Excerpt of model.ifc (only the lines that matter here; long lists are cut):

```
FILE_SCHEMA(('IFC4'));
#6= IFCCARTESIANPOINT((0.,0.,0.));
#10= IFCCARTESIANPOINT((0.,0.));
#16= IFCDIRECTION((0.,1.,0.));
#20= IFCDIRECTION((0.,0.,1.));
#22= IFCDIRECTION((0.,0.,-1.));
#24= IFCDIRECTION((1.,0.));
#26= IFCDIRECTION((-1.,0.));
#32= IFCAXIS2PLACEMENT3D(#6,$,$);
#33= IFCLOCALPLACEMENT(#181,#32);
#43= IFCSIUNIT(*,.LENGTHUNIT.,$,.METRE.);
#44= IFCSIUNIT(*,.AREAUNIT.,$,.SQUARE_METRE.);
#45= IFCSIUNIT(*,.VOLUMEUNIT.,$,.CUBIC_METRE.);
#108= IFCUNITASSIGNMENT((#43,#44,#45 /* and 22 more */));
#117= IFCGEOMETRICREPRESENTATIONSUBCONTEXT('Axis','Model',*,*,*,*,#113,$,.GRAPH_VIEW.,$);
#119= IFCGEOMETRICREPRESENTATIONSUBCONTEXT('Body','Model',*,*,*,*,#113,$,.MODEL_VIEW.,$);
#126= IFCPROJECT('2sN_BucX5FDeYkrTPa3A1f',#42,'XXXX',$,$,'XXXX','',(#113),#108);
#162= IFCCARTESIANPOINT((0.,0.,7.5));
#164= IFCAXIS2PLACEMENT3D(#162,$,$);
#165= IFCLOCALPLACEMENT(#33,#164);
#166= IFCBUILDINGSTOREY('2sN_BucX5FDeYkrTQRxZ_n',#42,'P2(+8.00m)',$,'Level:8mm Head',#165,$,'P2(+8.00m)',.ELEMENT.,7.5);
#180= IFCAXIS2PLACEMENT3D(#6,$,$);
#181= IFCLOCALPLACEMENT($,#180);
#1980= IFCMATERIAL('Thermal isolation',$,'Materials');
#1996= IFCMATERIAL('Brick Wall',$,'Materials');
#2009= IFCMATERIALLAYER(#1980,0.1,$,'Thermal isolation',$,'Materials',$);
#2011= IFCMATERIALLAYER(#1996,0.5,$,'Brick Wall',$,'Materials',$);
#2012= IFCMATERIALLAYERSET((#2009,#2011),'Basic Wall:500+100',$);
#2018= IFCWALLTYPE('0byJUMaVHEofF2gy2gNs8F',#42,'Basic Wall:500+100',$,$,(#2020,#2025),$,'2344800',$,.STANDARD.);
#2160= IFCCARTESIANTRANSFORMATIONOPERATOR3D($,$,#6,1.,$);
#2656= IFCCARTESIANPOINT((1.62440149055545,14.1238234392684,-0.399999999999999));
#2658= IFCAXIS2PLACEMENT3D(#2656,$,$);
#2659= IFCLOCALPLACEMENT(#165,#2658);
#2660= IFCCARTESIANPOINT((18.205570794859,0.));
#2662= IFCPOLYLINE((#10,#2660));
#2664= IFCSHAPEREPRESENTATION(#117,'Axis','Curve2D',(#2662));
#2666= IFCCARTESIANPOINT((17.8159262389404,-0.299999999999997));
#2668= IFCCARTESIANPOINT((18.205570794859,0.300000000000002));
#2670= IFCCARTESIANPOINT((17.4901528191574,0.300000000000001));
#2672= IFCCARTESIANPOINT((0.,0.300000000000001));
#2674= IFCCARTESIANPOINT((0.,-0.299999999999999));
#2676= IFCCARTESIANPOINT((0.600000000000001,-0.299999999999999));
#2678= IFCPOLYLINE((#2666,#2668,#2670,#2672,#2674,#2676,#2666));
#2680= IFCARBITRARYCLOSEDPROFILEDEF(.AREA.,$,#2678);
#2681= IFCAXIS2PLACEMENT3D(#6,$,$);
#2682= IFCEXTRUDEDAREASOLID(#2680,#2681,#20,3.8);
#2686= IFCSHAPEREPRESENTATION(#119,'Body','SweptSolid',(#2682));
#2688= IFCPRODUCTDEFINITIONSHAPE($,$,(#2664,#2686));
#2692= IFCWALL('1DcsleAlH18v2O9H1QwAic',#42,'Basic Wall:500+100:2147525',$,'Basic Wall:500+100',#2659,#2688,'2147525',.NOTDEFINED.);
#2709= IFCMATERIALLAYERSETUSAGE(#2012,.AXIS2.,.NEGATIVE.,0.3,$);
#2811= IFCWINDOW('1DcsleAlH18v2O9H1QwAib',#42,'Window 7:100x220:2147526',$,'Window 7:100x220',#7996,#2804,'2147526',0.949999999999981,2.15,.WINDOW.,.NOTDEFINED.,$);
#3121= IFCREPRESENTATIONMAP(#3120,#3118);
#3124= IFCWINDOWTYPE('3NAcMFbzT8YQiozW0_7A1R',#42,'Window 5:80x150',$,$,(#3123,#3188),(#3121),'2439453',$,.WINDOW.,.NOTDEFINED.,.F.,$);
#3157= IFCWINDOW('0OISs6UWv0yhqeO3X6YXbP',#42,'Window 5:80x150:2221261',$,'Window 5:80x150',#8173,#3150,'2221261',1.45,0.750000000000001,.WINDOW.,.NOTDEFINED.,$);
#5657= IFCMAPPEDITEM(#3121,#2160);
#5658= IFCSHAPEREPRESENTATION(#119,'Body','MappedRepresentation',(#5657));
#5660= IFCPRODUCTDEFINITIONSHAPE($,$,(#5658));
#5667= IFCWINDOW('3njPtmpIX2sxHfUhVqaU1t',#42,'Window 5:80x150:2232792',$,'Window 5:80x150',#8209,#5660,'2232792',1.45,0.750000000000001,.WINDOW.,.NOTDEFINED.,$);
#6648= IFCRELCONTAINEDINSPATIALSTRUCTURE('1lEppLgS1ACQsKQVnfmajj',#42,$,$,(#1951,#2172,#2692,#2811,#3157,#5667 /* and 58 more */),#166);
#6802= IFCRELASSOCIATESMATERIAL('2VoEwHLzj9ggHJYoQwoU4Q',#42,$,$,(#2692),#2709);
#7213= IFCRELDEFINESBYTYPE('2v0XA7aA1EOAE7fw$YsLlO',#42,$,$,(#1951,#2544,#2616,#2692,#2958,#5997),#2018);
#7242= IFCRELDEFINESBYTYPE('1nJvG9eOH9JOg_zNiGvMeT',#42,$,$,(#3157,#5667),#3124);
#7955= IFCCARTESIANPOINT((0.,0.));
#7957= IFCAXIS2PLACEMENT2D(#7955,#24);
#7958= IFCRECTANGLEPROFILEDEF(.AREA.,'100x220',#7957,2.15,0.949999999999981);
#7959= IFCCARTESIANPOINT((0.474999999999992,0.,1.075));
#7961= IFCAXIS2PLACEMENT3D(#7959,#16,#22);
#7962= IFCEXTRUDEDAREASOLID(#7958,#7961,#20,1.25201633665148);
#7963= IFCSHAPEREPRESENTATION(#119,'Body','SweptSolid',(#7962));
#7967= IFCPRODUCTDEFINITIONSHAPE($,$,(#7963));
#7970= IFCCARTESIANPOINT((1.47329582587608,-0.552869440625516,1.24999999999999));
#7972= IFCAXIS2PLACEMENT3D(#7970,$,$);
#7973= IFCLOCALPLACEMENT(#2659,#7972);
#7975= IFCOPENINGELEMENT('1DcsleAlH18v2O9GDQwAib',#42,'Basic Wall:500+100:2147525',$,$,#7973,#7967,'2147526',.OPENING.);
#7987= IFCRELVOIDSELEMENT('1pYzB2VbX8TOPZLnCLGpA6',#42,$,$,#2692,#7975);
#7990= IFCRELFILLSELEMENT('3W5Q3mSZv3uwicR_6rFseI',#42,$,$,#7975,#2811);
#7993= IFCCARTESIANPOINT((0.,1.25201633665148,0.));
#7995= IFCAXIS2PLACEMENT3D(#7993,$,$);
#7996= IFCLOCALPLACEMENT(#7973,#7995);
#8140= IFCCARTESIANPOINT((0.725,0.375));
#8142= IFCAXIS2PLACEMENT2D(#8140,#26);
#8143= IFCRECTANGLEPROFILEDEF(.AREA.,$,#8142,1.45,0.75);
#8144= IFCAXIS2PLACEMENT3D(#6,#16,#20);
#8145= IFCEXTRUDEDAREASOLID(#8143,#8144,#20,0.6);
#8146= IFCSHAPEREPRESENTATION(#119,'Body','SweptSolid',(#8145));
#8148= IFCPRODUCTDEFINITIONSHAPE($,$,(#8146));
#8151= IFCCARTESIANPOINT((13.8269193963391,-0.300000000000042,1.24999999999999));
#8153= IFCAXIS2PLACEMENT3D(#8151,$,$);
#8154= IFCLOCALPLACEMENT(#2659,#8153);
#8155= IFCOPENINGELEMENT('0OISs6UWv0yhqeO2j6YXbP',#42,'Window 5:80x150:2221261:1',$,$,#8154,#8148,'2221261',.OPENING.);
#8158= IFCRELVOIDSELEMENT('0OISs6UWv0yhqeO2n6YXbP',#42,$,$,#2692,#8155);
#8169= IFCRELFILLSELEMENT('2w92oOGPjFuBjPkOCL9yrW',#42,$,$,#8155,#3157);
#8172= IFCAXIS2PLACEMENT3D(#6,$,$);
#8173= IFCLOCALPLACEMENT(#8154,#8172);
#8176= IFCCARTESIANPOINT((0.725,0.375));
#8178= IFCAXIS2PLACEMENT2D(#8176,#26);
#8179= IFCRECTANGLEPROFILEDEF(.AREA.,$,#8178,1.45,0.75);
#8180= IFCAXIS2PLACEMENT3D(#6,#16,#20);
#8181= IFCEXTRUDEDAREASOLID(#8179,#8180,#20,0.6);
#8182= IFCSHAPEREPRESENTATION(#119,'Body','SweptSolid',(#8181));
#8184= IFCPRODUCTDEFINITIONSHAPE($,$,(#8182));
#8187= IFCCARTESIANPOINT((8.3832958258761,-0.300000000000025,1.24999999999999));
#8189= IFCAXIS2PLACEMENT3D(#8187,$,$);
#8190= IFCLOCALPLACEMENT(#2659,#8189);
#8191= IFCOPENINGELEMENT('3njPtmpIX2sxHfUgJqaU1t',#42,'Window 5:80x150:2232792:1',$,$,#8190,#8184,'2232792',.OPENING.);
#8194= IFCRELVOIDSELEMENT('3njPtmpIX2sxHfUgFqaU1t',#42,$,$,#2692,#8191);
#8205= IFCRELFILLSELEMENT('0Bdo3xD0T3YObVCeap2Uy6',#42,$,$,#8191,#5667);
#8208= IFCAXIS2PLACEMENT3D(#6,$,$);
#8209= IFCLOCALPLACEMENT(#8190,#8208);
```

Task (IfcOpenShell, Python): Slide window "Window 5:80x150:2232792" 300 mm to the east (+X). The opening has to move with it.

```python
import ifcopenshell
import ifcopenshell.api.geometry
import ifcopenshell.util.placement

model = ifcopenshell.open("model.ifc")

window = model.by_id(5667)
opening = window.FillsVoids[0].RelatingOpeningElement
wall = opening.VoidsElements[0].RelatingBuildingElement

wall_matrix = ifcopenshell.util.placement.get_local_placement(wall.ObjectPlacement)
shift = wall_matrix[:3, 0] * 0.3
before = ifcopenshell.util.placement.get_local_placement(window.ObjectPlacement)[:3, 3].copy()

# The window is placed relative to its opening, so it follows when the opening moves.
matrix = ifcopenshell.util.placement.get_local_placement(opening.ObjectPlacement)
matrix[:3, 3] += shift
ifcopenshell.api.geometry.edit_object_placement(
    model, product=opening, matrix=matrix, is_si=False, should_transform_children=True
)

after = ifcopenshell.util.placement.get_local_placement(window.ObjectPlacement)[:3, 3]
print("window moved by", (after - before).round(3) + 0.0)

model.write("model_rev.ifc")
```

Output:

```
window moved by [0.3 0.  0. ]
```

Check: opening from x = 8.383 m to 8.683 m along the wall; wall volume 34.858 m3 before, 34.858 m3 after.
